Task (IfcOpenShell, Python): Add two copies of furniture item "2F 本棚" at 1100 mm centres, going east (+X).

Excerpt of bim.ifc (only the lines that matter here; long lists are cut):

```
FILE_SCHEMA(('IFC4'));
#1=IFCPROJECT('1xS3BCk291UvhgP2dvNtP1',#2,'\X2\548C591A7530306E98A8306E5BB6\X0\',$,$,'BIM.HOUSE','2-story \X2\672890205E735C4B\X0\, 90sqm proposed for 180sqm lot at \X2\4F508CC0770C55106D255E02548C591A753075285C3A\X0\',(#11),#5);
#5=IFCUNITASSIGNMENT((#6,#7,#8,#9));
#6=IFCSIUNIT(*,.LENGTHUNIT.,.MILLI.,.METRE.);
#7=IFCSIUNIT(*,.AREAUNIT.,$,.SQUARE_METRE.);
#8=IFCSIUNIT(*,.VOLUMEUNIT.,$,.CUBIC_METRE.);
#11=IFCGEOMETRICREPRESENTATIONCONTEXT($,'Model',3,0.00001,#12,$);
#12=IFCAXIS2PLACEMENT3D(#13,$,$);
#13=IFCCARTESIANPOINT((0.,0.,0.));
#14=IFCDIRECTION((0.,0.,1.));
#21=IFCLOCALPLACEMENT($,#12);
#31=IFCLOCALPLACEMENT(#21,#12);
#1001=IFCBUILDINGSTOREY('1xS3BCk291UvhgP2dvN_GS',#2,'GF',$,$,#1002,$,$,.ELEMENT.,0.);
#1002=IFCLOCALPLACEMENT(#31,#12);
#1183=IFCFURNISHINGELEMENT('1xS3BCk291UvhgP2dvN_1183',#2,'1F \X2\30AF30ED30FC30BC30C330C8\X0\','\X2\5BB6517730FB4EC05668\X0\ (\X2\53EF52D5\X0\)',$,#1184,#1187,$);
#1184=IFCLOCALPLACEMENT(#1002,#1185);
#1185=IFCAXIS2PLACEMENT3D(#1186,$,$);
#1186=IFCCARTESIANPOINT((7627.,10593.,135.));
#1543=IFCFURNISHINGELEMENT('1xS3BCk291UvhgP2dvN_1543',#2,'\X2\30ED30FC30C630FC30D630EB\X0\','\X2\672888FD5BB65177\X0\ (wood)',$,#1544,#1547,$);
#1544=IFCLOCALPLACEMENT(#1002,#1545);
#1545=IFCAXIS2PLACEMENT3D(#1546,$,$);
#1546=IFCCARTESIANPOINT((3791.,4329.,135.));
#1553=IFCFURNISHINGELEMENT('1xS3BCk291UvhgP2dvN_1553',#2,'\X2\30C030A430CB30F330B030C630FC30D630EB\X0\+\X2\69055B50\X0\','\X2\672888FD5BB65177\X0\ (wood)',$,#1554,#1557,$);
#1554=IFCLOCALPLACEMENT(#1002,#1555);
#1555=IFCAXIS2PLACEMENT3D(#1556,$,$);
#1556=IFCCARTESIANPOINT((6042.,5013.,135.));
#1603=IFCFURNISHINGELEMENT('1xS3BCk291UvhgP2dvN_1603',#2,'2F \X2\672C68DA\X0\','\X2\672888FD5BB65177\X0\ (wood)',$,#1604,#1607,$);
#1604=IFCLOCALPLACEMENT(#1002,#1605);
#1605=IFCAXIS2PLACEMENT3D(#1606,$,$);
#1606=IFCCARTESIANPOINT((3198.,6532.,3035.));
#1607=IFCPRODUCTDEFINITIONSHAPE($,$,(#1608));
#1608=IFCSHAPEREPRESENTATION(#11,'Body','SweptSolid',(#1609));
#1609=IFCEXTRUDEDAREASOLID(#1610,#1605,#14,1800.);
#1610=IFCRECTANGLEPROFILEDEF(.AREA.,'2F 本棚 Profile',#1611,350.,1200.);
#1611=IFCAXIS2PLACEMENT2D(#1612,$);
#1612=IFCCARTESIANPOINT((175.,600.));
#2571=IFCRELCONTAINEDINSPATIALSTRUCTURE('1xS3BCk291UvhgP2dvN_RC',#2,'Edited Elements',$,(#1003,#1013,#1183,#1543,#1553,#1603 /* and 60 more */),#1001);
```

```python
import numpy as np
import ifcopenshell
import ifcopenshell.api.geometry
import ifcopenshell.api.root
import ifcopenshell.util.element
import ifcopenshell.util.placement

model = ifcopenshell.open("bim.ifc")


def reuse_history(source, copy):
    """copy_class also copies each property set's owner history, people and application; keep the originals."""
    for rel in copy.IsDefinedBy:
        if rel.is_a("IfcRelDefinesByProperties") and (history := rel.RelatingPropertyDefinition.OwnerHistory):
            rel.RelatingPropertyDefinition.OwnerHistory = source.OwnerHistory
            ifcopenshell.util.element.remove_deep2(model, history)


source = model.by_id(1603)
base = ifcopenshell.util.placement.get_local_placement(source.ObjectPlacement)
step = np.array([1.0, 0.0, 0.0]) * 1100.0

for i in range(1, 3):
    copy = ifcopenshell.api.root.copy_class(model, product=source)
    copy.Representation = ifcopenshell.util.element.copy_deep(
        model, source.Representation, exclude=["IfcGeometricRepresentationContext", "IfcRepresentationMap"]
    )
    reuse_history(source, copy)
    matrix = base.copy()
    matrix[:3, 3] += i * step
    print("added at", matrix[:3, 3].round(3) + 0.0)
    ifcopenshell.api.geometry.edit_object_placement(model, product=copy, matrix=matrix, is_si=False)

model.write("bim_v2.ifc")
```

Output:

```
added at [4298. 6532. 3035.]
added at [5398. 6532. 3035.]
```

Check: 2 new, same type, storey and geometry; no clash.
